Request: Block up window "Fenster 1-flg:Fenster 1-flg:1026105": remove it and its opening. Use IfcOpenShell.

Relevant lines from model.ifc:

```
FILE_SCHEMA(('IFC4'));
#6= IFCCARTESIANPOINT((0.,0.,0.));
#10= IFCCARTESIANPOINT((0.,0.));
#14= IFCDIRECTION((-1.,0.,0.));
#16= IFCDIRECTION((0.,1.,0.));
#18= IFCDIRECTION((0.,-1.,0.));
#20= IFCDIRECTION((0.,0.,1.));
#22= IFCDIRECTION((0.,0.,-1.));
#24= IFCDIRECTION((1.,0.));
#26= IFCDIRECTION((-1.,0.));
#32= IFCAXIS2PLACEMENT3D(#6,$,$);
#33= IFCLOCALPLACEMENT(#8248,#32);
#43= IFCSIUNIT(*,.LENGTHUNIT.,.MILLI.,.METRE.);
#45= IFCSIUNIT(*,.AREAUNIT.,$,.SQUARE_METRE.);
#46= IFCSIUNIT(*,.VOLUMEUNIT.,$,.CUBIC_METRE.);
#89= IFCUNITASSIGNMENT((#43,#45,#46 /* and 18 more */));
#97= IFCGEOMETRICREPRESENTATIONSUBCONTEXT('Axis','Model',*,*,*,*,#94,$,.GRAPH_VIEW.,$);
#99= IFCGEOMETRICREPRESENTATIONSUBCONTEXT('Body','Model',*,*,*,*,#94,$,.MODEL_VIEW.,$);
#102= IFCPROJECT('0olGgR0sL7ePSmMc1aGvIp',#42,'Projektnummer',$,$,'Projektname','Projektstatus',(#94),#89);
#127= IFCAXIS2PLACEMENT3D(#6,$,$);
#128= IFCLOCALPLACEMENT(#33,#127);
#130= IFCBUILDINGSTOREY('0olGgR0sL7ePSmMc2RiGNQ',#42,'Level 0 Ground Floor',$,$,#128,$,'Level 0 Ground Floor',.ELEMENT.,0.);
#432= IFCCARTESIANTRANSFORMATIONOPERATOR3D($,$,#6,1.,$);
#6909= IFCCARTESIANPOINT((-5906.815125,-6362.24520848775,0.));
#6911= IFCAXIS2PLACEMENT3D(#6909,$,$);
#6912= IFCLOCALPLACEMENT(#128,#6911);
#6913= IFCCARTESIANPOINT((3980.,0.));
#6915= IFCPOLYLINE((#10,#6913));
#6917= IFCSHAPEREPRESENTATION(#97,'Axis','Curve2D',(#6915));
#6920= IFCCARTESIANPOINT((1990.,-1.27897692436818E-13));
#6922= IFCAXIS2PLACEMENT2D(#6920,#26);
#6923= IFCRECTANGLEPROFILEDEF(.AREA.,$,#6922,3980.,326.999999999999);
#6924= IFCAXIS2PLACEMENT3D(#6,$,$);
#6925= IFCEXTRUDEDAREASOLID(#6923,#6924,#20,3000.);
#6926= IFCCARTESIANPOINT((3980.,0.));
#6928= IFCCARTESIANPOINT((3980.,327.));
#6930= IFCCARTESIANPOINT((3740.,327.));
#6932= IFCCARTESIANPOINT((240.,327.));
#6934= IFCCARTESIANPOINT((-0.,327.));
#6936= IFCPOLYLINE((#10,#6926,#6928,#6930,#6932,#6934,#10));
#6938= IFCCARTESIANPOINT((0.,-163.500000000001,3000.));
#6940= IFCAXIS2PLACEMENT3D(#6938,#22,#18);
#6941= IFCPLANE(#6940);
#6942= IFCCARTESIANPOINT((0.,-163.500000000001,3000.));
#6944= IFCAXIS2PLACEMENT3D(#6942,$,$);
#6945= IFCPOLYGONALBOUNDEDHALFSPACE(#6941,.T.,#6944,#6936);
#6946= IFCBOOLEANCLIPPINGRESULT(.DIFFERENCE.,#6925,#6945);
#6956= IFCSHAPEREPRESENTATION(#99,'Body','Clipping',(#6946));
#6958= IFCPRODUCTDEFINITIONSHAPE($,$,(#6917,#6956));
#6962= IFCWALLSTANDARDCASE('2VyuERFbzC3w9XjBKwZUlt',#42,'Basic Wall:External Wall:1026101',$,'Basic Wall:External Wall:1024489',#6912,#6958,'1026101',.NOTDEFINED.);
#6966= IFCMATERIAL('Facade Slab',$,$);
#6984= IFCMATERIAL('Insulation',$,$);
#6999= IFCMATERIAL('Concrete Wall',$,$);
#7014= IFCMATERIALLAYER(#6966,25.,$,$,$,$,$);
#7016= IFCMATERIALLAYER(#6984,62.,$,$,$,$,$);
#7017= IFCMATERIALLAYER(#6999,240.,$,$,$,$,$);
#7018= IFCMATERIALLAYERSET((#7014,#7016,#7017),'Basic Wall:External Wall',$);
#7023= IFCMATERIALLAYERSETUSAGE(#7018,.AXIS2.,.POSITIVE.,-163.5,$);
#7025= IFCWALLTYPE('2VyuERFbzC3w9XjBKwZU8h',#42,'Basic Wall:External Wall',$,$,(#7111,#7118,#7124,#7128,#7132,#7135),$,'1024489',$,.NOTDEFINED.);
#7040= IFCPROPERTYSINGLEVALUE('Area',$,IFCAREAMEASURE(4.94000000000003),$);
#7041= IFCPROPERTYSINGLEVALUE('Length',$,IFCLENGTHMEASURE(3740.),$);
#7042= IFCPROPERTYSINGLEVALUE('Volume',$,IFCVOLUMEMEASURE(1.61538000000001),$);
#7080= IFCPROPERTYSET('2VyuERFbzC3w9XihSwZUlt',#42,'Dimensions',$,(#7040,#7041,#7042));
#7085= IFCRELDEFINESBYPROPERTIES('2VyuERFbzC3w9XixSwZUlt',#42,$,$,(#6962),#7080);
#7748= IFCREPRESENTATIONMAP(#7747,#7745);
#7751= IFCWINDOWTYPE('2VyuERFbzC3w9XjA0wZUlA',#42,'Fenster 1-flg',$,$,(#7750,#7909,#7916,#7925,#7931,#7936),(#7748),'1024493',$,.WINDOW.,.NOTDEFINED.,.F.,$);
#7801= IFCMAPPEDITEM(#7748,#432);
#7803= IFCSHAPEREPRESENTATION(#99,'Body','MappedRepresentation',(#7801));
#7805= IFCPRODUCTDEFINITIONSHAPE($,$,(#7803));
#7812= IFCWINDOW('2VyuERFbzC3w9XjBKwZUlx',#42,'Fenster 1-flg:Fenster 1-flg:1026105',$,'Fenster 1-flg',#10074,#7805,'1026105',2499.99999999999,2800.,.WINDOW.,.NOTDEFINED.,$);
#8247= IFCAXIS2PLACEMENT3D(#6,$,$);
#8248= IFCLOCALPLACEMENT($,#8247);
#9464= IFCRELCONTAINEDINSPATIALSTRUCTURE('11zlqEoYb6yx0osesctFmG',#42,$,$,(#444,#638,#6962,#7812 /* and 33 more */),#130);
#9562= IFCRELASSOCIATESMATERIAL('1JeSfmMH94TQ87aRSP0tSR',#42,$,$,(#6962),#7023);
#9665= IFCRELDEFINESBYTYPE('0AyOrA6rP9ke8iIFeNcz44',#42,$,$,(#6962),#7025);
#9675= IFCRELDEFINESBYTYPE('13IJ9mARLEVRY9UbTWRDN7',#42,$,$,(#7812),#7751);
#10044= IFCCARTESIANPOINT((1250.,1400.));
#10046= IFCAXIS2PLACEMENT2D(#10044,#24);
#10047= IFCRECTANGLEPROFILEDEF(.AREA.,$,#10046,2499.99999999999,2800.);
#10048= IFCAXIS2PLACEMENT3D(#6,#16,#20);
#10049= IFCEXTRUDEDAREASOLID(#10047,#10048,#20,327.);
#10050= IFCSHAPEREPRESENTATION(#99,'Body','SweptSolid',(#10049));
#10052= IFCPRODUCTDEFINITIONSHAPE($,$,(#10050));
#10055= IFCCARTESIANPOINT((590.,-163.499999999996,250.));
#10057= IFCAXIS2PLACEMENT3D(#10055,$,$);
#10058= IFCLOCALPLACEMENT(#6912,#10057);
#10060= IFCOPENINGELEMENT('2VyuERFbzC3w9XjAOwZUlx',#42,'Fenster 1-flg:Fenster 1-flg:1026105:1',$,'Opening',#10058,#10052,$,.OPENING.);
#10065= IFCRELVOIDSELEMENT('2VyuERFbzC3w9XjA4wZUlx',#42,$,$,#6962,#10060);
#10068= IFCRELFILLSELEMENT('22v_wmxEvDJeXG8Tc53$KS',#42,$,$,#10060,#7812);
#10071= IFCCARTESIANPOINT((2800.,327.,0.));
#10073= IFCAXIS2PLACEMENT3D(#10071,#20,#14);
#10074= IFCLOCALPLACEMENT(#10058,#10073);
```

```python
import ifcopenshell
import ifcopenshell.api.feature
import ifcopenshell.api.pset
import ifcopenshell.api.root
import ifcopenshell.geom
import ifcopenshell.util.element
import ifcopenshell.util.shape
import ifcopenshell.util.unit

model = ifcopenshell.open("model.ifc")
area_scale = ifcopenshell.util.unit.calculate_unit_scale(model, "AREAUNIT")
volume_scale = ifcopenshell.util.unit.calculate_unit_scale(model, "VOLUMEUNIT")
settings = ifcopenshell.geom.settings()


def volume(element):
    """Net volume in cubic metres, openings subtracted."""
    shape = ifcopenshell.geom.create_shape(settings, element)
    return ifcopenshell.util.shape.get_volume(shape.geometry)


window = model.by_guid("2VyuERFbzC3w9XjBKwZUlx")
opening = window.FillsVoids[0].RelatingOpeningElement
wall = opening.VoidsElements[0].RelatingBuildingElement
before = volume(wall)

ifcopenshell.api.root.remove_product(model, product=window)
ifcopenshell.api.feature.remove_feature(model, feature=opening)

after = volume(wall)
thickness = 0.327  # wall thickness in metres

# Update the wall's stored quantities.
pset = model.by_id(ifcopenshell.util.element.get_pset(wall, "Dimensions", should_inherit=False)["id"])
ifcopenshell.api.pset.edit_pset(model, pset=pset, properties={
    "Area": model.create_entity("IfcAreaMeasure", after / thickness / area_scale),
    "Volume": model.create_entity("IfcVolumeMeasure", after / volume_scale),
})

print(f"wall volume {before:.3f} -> {after:.3f} m3")

model.write("model-out.ifc")
```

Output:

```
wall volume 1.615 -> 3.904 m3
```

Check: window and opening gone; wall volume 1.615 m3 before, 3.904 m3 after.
